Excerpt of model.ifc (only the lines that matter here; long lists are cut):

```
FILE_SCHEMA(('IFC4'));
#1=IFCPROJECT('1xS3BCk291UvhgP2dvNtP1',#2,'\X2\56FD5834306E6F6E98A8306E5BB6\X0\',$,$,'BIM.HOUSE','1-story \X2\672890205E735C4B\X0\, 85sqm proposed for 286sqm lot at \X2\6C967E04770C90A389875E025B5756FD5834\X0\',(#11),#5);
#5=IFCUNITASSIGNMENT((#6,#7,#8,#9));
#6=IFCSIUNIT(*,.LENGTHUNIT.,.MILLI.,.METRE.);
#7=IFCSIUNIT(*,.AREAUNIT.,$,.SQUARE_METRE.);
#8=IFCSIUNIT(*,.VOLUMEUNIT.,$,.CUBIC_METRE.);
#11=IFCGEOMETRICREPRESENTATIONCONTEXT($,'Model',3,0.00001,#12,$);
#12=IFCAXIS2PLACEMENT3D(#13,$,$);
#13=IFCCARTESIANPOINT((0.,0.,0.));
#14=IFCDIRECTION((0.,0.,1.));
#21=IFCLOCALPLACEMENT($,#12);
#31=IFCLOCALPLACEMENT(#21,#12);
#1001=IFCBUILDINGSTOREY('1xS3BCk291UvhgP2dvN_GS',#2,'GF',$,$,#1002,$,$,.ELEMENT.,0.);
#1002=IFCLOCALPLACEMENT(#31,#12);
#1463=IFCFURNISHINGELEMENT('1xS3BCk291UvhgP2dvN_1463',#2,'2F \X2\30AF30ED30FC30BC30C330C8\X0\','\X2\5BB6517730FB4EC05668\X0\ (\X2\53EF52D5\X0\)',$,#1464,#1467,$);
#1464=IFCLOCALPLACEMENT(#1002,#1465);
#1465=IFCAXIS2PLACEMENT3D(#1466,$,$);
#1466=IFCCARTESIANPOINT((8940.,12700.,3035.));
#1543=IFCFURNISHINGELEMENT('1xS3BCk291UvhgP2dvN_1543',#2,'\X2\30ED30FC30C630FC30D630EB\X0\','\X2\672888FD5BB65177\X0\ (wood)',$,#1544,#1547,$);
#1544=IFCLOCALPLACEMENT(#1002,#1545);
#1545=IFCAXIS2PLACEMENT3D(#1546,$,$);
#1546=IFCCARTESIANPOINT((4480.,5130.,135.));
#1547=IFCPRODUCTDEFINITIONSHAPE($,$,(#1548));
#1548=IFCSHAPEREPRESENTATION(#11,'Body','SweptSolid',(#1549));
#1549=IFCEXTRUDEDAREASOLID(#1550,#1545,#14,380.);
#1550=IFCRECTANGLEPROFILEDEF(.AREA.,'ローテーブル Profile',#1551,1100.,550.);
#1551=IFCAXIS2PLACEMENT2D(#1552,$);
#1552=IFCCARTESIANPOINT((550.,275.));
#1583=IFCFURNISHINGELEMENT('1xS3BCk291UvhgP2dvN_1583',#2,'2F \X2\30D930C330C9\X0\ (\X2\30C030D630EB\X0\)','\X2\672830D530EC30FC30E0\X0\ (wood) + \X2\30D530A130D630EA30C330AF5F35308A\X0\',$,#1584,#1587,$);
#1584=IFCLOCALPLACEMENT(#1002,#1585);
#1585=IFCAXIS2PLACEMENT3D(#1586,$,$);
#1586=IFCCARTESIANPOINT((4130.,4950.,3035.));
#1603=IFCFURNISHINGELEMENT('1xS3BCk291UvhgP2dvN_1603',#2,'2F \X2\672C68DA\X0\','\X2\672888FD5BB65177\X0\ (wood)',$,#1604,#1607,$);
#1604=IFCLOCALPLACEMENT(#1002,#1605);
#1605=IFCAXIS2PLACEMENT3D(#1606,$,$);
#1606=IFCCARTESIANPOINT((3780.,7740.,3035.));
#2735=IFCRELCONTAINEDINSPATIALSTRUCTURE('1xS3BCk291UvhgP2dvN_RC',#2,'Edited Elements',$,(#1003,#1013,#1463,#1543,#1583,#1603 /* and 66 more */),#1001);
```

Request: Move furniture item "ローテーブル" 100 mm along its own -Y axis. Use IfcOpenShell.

```python
import ifcopenshell
import ifcopenshell.api.geometry
import ifcopenshell.util.placement
import ifcopenshell.util.unit

model = ifcopenshell.open("model.ifc")
unit_scale = ifcopenshell.util.unit.calculate_unit_scale(model)

item = model.by_guid("1xS3BCk291UvhgP2dvN_1543")
matrix = ifcopenshell.util.placement.get_local_placement(item.ObjectPlacement)
matrix[:3, 3] -= matrix[:3, 1] * 0.1 / unit_scale
ifcopenshell.api.geometry.edit_object_placement(model, product=item, matrix=matrix, is_si=False)

print(ifcopenshell.util.placement.get_local_placement(item.ObjectPlacement).round(3) + 0.0)

model.write("model_v2.ifc")
```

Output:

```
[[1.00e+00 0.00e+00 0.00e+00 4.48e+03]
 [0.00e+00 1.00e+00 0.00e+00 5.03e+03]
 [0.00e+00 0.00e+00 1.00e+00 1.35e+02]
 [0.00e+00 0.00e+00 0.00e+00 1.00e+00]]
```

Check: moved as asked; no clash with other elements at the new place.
